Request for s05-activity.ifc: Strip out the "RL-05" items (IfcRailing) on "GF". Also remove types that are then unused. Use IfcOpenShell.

First a look at what the model holds.

```python
import ifcopenshell
import ifcopenshell.util.element

model = ifcopenshell.open("s05-activity.ifc")
print(model.schema)
storey = next(s for s in model.by_type("IfcBuildingStorey") if s.Name == "GF")
railings = [e for e in ifcopenshell.util.element.get_decomposition(storey) if e.is_a("IfcRailing")]
seen = {}
for e in railings:
    element_type = ifcopenshell.util.element.get_type(e)
    name = element_type.Name if element_type not in (None, e) else None
    seen[name] = seen.get(name, 0) + 1
for name, count in sorted(seen.items(), key=str):
    print(count, "x", name)
```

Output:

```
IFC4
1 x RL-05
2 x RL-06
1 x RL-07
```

```python
import ifcopenshell
import ifcopenshell.api.root
import ifcopenshell.util.element

model = ifcopenshell.open("s05-activity.ifc")

storey = next(s for s in model.by_type("IfcBuildingStorey") if s.Name == "GF")
railings = [e for e in ifcopenshell.util.element.get_decomposition(storey) if e.is_a("IfcRailing")]
targets = [e for e in railings if (t := ifcopenshell.util.element.get_type(e)) not in (None, e) and t.Name == "RL-05"]
types = {ifcopenshell.util.element.get_type(e) for e in targets} - {None, *targets}

for e in targets:
    ifcopenshell.api.root.remove_product(model, product=e)
print(len(targets), "removed")

unused = [t for t in types if not ifcopenshell.util.element.get_types(t)]
for t in unused:
    ifcopenshell.api.root.remove_product(model, product=t)
print(len(unused), "unused types removed")

model.write("s05-activity_v2.ifc")
```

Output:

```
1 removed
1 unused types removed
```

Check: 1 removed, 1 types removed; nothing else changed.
